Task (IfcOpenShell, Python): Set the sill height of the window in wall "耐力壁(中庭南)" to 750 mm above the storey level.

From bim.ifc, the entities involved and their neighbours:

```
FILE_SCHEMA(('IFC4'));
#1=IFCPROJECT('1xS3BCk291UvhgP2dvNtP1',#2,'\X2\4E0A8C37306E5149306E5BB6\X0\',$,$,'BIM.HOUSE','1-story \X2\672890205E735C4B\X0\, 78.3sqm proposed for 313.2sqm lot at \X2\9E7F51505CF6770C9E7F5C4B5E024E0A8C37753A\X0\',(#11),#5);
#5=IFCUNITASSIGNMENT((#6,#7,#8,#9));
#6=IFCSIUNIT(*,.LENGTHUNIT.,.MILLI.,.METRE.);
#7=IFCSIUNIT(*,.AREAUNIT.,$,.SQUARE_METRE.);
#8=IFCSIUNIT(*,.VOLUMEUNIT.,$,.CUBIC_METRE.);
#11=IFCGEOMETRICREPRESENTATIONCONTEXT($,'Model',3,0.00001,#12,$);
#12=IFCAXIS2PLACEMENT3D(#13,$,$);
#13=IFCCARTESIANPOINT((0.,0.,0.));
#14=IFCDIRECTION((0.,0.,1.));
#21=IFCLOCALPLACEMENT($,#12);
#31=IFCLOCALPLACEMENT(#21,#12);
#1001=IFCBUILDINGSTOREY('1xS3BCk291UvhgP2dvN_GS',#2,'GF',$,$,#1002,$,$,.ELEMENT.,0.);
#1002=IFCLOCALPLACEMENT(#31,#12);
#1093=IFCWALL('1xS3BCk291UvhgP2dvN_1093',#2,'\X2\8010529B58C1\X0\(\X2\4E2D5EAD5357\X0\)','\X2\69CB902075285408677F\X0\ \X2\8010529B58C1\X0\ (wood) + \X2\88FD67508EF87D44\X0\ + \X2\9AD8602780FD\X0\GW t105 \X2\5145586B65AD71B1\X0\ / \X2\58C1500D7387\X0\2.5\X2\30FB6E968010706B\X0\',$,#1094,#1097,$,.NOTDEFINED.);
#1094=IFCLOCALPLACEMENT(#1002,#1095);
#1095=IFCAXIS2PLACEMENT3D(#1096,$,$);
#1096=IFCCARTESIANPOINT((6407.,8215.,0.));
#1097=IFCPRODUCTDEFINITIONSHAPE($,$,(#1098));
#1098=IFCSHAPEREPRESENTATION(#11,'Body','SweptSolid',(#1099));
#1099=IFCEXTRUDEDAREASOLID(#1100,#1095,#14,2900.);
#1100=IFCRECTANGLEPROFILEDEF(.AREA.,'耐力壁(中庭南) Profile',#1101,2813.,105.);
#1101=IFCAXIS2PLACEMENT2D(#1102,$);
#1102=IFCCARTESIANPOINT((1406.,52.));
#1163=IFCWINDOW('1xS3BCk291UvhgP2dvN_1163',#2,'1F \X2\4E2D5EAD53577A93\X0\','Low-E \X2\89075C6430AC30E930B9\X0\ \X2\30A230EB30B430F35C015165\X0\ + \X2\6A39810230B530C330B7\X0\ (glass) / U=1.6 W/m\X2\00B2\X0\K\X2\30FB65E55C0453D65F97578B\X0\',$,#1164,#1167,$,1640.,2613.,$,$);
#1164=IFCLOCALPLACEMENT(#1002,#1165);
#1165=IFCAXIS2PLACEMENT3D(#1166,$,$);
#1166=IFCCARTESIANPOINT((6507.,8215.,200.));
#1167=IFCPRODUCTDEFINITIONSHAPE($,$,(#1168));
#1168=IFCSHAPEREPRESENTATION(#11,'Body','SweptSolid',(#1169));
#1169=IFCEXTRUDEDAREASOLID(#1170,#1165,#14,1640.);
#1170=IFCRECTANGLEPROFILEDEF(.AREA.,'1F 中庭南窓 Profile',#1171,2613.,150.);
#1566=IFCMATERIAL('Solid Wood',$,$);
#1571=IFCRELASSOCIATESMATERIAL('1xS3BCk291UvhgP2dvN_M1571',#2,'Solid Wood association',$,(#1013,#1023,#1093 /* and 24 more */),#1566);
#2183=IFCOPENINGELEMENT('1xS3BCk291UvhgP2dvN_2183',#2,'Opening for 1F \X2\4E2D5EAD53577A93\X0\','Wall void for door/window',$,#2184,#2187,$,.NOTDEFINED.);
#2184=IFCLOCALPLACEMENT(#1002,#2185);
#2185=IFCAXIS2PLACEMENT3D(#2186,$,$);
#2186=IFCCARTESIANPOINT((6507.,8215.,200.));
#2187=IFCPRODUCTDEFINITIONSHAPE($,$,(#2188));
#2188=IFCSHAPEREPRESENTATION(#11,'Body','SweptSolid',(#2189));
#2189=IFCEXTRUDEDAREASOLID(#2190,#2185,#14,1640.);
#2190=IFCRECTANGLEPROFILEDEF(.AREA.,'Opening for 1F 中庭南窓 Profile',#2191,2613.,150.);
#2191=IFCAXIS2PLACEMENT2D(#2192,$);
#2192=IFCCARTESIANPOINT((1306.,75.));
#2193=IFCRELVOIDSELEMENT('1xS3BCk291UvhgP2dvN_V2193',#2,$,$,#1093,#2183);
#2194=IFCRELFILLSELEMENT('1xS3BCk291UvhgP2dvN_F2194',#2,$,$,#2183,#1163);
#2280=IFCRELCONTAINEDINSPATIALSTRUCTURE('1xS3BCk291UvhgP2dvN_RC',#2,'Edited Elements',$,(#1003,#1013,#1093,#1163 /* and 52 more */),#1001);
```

```python
import numpy as np
import ifcopenshell
import ifcopenshell.api.geometry
import ifcopenshell.geom
import ifcopenshell.util.element
import ifcopenshell.util.placement
import ifcopenshell.util.shape
import ifcopenshell.util.unit

model = ifcopenshell.open("bim.ifc")
unit_scale = ifcopenshell.util.unit.calculate_unit_scale(model)

window = model.by_guid("1xS3BCk291UvhgP2dvN_1163")
opening = window.FillsVoids[0].RelatingOpeningElement
storey = ifcopenshell.util.element.get_container(window, ifc_class="IfcBuildingStorey")
level = ifcopenshell.util.placement.get_local_placement(storey.ObjectPlacement)[2, 3]

# The opening's origin need not be at the sill, so measure its lowest point.
shape = ifcopenshell.geom.create_shape(ifcopenshell.geom.settings(), opening)
bottom = ifcopenshell.util.shape.get_shape_bottom_elevation(shape, shape.geometry) / unit_scale
dz = level + 0.75 / unit_scale - bottom

shift = np.array([0.0, 0.0, dz])
# The window is not placed relative to its opening, so move both.
for product in (opening, window):
    matrix = ifcopenshell.util.placement.get_local_placement(product.ObjectPlacement)
    matrix[:3, 3] += shift
    ifcopenshell.api.geometry.edit_object_placement(model, product=product, matrix=matrix, is_si=False)

print(f"moved by {dz * unit_scale:+.3f} m")

model.write("bim_v2.ifc")
```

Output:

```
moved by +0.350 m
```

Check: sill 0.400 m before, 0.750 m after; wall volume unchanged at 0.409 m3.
